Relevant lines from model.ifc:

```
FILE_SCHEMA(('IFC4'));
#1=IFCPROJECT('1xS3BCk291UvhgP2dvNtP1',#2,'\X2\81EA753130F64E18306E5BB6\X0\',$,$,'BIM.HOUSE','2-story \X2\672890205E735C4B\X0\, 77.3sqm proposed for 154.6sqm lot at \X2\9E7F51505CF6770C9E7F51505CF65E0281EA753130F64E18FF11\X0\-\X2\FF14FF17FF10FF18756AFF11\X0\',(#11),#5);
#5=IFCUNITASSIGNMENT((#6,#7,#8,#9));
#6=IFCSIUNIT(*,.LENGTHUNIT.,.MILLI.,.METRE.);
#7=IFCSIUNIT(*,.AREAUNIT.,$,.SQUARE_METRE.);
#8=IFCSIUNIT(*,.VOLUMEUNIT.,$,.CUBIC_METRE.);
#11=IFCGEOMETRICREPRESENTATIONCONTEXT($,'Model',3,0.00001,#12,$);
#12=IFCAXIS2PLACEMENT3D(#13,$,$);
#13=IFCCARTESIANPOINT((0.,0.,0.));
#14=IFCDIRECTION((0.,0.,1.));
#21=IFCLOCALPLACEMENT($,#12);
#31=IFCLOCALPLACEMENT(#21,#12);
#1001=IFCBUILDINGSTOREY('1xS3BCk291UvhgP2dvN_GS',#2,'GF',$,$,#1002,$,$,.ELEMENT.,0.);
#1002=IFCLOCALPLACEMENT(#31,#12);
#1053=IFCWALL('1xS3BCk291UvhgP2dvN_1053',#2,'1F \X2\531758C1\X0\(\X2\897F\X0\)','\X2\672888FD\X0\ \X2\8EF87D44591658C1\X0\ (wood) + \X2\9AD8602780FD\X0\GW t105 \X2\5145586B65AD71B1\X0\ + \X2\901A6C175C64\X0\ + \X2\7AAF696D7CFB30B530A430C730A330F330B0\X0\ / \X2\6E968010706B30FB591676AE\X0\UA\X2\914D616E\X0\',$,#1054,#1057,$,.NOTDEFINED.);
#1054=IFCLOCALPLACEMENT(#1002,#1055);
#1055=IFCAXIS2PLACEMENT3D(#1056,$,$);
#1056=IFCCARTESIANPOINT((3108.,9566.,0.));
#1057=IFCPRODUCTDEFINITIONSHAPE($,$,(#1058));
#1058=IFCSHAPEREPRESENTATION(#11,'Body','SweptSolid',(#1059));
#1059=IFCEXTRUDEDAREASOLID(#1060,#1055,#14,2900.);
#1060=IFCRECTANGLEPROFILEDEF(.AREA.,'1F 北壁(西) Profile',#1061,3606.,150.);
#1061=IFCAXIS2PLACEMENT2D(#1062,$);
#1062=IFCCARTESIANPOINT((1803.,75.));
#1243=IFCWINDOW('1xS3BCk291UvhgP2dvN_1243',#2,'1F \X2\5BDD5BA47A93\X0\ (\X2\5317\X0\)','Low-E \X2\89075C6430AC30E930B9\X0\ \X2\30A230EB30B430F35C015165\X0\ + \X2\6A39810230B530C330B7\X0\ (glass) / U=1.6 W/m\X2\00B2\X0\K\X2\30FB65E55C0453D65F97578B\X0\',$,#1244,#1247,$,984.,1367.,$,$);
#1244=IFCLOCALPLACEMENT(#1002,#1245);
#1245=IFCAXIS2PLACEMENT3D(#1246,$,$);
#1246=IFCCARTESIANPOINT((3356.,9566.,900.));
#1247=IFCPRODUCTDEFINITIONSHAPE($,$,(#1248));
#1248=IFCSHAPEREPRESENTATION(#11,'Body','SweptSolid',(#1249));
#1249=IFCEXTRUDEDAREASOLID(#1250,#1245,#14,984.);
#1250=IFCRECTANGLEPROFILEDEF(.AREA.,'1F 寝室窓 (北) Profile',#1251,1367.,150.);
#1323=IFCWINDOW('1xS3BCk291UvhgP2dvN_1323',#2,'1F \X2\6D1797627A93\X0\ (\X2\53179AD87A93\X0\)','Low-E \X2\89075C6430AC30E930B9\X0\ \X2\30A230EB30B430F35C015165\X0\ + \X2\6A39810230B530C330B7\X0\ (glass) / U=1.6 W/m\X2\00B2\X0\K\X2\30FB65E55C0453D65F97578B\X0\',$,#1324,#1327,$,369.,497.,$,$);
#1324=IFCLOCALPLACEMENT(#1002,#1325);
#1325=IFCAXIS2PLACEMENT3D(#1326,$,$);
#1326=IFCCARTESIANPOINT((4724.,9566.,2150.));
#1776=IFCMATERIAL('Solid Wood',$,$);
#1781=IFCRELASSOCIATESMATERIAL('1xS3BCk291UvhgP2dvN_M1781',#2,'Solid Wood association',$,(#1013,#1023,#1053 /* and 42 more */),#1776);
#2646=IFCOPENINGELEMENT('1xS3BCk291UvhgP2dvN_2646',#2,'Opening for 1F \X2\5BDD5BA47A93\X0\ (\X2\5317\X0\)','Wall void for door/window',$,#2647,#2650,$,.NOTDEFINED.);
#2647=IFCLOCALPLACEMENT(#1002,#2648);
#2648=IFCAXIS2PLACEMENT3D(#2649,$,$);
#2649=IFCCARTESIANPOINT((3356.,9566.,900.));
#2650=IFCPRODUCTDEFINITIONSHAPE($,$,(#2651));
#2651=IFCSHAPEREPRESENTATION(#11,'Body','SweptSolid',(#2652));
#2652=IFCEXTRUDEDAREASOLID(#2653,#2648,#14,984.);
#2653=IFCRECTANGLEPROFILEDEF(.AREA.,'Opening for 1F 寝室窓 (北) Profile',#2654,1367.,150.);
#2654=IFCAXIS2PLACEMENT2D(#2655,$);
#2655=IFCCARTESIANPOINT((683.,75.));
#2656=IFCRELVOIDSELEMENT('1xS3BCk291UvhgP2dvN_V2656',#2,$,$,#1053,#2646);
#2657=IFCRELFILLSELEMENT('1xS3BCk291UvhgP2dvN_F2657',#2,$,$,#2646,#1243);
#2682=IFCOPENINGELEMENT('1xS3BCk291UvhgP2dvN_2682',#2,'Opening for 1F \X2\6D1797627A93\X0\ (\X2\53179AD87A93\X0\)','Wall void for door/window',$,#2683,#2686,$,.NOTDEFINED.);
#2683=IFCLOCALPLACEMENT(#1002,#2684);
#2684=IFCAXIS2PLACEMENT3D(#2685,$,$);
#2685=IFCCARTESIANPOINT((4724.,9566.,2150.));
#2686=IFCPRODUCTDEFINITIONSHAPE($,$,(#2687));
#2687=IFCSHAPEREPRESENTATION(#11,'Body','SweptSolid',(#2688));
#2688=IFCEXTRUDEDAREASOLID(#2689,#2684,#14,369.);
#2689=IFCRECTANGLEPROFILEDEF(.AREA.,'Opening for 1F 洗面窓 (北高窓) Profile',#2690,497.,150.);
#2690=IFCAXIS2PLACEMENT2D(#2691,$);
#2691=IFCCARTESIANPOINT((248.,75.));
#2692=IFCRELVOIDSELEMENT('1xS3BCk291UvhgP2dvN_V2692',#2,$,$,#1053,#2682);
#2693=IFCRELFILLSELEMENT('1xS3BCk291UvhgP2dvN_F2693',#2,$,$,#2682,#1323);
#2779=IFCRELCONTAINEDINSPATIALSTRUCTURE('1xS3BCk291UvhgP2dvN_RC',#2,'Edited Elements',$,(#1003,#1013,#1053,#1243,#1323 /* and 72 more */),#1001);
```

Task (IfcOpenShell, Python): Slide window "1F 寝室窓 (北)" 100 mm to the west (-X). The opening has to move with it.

```python
import ifcopenshell
import ifcopenshell.api.geometry
import ifcopenshell.util.placement
import ifcopenshell.util.unit

model = ifcopenshell.open("model.ifc")
unit_scale = ifcopenshell.util.unit.calculate_unit_scale(model)

window = model.by_guid("1xS3BCk291UvhgP2dvN_1243")
opening = window.FillsVoids[0].RelatingOpeningElement
wall = opening.VoidsElements[0].RelatingBuildingElement

wall_matrix = ifcopenshell.util.placement.get_local_placement(wall.ObjectPlacement)
shift = wall_matrix[:3, 0] * -0.1 / unit_scale
before = ifcopenshell.util.placement.get_local_placement(window.ObjectPlacement)[:3, 3].copy()

# The window is not placed relative to its opening, so move both.
for product in (opening, window):
    matrix = ifcopenshell.util.placement.get_local_placement(product.ObjectPlacement)
    matrix[:3, 3] += shift
    ifcopenshell.api.geometry.edit_object_placement(model, product=product, matrix=matrix, is_si=False)

after = ifcopenshell.util.placement.get_local_placement(window.ObjectPlacement)[:3, 3]
print("window moved by", (after - before).round(3) + 0.0)

model.write("model_updated.ifc")
```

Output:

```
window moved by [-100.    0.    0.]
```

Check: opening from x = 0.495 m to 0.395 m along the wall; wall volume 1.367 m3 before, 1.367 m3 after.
